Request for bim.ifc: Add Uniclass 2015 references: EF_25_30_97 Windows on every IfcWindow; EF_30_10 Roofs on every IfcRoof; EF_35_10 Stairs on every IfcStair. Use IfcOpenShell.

First a look at what the model holds.

```python
import ifcopenshell

model = ifcopenshell.open("bim.ifc")
print(model.schema)
print("classifications:", [c.Name for c in model.by_type("IfcClassification")])
for ifc_class in ("IfcDoor", "IfcRoof", "IfcStair", "IfcWall", "IfcWindow"):
    print(ifc_class, len(model.by_type(ifc_class)))
```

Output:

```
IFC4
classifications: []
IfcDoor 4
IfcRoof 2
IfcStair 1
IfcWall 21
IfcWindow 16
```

```python
import ifcopenshell
import ifcopenshell.api.classification

model = ifcopenshell.open("bim.ifc")

system = ifcopenshell.api.classification.add_classification(model, classification="Uniclass 2015")

codes = {
    "IfcWindow": ("EF_25_30_97", "Windows"),
    "IfcRoof": ("EF_30_10", "Roofs"),
    "IfcStair": ("EF_35_10", "Stairs"),
}
for ifc_class, (code, name) in codes.items():
    products = model.by_type(ifc_class)
    ifcopenshell.api.classification.add_reference(
        model, products=products, classification=system, identification=code, name=name
    )
    print(code, len(products))

model.write("bim_v2.ifc")
```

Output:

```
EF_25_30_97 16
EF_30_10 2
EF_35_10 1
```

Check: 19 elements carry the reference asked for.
